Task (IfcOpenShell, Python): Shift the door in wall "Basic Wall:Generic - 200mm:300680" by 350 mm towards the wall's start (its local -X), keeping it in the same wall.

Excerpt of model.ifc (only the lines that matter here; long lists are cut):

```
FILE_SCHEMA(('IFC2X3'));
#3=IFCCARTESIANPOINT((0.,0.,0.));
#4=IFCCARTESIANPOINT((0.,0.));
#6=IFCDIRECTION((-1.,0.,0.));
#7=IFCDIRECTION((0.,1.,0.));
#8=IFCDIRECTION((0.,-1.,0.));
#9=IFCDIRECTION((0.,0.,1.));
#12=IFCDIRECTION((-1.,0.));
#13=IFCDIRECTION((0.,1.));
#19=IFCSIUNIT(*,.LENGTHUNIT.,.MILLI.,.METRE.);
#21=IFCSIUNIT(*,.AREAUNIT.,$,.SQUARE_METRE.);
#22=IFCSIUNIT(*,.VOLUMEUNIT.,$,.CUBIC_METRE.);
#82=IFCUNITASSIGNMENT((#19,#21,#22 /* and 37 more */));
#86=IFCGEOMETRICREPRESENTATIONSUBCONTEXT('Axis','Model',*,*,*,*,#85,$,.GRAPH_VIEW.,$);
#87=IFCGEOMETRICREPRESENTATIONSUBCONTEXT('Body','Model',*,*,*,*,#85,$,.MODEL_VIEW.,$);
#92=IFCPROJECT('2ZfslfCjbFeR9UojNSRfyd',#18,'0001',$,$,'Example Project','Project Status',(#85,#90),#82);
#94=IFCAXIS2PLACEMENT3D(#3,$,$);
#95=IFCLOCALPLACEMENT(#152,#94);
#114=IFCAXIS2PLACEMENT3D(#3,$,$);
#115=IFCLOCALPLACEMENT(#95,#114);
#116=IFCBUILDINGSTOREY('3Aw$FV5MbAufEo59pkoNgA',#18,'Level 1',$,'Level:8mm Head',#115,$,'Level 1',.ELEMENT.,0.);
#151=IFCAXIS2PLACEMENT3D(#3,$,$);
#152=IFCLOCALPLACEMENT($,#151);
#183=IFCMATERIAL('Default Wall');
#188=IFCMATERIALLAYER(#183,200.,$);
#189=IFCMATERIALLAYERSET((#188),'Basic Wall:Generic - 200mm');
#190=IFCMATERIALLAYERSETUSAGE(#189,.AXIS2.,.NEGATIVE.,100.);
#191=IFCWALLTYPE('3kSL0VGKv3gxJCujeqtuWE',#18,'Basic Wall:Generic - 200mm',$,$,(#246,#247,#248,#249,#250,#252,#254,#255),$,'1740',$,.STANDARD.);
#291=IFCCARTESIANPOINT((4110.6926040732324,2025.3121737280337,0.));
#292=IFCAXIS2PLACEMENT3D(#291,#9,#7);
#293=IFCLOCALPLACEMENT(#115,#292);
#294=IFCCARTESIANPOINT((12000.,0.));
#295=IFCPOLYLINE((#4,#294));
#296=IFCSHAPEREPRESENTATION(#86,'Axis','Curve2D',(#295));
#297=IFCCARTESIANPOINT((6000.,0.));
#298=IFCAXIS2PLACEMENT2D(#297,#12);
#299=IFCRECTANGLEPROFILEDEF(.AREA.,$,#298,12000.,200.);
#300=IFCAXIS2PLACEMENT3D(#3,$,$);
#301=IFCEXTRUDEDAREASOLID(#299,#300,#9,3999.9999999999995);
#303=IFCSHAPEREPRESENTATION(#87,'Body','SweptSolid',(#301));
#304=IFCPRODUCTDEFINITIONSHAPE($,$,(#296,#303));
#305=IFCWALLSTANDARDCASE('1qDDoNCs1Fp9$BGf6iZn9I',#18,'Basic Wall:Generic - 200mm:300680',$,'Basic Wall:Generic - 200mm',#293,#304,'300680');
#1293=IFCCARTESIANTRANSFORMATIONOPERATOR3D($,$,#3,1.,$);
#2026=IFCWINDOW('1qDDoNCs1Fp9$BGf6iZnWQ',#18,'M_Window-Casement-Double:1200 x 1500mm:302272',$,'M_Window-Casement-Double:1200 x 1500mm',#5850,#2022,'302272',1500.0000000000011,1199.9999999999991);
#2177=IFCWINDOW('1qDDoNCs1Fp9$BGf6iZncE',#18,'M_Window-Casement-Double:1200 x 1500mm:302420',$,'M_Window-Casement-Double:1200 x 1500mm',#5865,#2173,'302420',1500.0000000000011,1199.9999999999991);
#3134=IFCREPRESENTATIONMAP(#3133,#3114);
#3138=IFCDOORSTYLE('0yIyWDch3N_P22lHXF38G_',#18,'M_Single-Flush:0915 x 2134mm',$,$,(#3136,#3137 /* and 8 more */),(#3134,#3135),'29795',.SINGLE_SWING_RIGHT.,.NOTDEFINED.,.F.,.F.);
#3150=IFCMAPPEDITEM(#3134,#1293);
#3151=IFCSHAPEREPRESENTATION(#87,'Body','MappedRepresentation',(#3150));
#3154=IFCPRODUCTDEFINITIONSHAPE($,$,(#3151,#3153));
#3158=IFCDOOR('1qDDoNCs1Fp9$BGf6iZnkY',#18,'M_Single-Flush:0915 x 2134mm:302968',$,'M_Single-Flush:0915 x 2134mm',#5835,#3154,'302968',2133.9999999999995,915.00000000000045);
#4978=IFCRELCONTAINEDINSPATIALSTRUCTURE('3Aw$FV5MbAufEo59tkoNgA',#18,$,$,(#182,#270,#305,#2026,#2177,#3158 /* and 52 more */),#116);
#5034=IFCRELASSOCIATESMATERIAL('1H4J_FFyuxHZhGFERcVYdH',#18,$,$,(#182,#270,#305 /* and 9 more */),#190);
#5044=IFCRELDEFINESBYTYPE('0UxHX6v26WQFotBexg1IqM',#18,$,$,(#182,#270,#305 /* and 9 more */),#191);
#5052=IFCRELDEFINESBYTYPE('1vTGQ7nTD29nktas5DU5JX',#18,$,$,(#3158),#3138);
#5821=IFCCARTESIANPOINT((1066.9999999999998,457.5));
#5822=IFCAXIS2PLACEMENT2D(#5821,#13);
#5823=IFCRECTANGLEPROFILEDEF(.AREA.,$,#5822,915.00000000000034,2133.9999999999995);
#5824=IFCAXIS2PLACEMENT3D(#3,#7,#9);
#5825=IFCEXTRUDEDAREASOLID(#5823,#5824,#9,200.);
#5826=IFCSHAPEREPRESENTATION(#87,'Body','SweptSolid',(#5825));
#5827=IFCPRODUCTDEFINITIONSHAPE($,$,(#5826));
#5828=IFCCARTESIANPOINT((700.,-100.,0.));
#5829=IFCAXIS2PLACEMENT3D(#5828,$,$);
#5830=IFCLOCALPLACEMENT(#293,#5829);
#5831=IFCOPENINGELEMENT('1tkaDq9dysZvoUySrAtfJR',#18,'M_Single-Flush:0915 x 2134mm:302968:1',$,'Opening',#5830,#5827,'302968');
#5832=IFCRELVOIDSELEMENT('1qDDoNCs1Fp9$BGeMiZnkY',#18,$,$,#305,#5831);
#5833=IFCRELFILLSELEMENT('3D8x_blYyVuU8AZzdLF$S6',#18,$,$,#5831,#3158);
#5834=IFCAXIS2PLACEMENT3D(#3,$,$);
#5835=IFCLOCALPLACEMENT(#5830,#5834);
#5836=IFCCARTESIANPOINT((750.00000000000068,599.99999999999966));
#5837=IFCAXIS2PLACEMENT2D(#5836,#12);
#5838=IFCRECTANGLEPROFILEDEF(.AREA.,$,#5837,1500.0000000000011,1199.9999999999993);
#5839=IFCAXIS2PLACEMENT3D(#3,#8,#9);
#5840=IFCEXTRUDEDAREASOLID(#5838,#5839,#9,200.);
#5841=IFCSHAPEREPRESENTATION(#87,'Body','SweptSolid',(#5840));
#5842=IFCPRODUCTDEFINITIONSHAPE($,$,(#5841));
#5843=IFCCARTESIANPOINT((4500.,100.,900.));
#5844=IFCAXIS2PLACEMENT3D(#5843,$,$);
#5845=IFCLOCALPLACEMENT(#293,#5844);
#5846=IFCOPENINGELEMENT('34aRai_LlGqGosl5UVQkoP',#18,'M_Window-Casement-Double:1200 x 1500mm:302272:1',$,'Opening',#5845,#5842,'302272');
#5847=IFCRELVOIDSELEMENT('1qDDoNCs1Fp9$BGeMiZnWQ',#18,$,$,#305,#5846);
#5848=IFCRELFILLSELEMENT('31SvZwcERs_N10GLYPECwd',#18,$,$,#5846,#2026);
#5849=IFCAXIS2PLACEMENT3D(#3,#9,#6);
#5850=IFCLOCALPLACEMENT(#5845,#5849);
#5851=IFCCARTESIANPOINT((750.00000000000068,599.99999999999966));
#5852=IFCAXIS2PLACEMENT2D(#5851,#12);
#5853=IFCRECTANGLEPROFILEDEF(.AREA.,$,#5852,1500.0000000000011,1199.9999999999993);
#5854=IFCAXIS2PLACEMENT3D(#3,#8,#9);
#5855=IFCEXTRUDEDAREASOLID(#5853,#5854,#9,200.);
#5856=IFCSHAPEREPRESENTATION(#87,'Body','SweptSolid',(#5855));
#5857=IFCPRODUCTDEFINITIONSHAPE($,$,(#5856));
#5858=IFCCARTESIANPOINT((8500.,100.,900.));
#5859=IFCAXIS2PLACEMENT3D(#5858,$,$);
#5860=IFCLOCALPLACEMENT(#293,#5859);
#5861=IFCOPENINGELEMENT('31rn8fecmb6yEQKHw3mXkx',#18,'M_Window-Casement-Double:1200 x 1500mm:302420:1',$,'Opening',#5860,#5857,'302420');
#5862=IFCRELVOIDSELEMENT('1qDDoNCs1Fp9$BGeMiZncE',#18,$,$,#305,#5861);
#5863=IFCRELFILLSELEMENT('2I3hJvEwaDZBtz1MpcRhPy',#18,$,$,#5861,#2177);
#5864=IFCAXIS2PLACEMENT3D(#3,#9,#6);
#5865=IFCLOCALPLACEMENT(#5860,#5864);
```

```python
import ifcopenshell
import ifcopenshell.api.geometry
import ifcopenshell.util.placement

model = ifcopenshell.open("model.ifc")

door = model.by_guid("1qDDoNCs1Fp9$BGf6iZnkY")
opening = door.FillsVoids[0].RelatingOpeningElement
wall = opening.VoidsElements[0].RelatingBuildingElement

wall_matrix = ifcopenshell.util.placement.get_local_placement(wall.ObjectPlacement)
shift = wall_matrix[:3, 0] * -350.0
before = ifcopenshell.util.placement.get_local_placement(door.ObjectPlacement)[:3, 3].copy()

# The door is placed relative to its opening, so it follows when the opening moves.
matrix = ifcopenshell.util.placement.get_local_placement(opening.ObjectPlacement)
matrix[:3, 3] += shift
ifcopenshell.api.geometry.edit_object_placement(
    model, product=opening, matrix=matrix, is_si=False, should_transform_children=True
)

after = ifcopenshell.util.placement.get_local_placement(door.ObjectPlacement)[:3, 3]
print("door moved by", (after - before).round(3) + 0.0)

model.write("model-out.ifc")
```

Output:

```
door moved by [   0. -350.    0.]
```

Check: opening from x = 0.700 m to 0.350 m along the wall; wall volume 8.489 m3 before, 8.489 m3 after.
